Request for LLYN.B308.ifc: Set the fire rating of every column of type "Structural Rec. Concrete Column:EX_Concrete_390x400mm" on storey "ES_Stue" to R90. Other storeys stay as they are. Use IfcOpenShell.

First a look at what the model holds.

```python
import ifcopenshell
import ifcopenshell.util.element

model = ifcopenshell.open("LLYN.B308.ifc")
print(model.schema)
storey = next(s for s in model.by_type("IfcBuildingStorey") if s.Name == "ES_Stue")
columns = [e for e in ifcopenshell.util.element.get_decomposition(storey) if e.is_a("IfcColumn")]
seen = {}
for e in columns:
    element_type = ifcopenshell.util.element.get_type(e)
    key = (element_type.Name if element_type != e and element_type else None, ifcopenshell.util.element.get_pset(e, "Pset_ColumnCommon", "FireRating"))
    seen[key] = seen.get(key, 0) + 1
for (name, value), count in sorted(seen.items(), key=str):
    print(count, "x", name, "|", value)
```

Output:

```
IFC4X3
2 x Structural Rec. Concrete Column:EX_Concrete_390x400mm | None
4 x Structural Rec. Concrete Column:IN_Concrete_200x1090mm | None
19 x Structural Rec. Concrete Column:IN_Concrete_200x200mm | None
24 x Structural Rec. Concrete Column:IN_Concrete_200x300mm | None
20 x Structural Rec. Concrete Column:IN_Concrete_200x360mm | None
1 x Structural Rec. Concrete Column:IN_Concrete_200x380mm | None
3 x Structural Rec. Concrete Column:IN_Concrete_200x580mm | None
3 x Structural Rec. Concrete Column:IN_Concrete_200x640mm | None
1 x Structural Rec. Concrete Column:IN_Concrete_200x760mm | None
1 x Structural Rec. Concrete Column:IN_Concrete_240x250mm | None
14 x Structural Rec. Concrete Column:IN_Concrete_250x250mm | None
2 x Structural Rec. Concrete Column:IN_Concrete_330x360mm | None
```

```python
import ifcopenshell
import ifcopenshell.api.pset
import ifcopenshell.util.element

model = ifcopenshell.open("LLYN.B308.ifc")

storey = next(s for s in model.by_type("IfcBuildingStorey") if s.Name == "ES_Stue")
columns = [e for e in ifcopenshell.util.element.get_decomposition(storey) if e.is_a("IfcColumn")]

count = 0
for e in columns:
    element_type = ifcopenshell.util.element.get_type(e)
    if element_type in (None, e) or element_type.Name != "Structural Rec. Concrete Column:EX_Concrete_390x400mm":
        continue
    # add_pset returns the element's existing set when there is one.
    pset = ifcopenshell.api.pset.add_pset(model, product=e, name="Pset_ColumnCommon")
    ifcopenshell.api.pset.edit_pset(model, pset=pset, properties={"FireRating": "R90"})
    count += 1

print(count, "columns updated")

model.write("LLYN.B308_v2.ifc")
```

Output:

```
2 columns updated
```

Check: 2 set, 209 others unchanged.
